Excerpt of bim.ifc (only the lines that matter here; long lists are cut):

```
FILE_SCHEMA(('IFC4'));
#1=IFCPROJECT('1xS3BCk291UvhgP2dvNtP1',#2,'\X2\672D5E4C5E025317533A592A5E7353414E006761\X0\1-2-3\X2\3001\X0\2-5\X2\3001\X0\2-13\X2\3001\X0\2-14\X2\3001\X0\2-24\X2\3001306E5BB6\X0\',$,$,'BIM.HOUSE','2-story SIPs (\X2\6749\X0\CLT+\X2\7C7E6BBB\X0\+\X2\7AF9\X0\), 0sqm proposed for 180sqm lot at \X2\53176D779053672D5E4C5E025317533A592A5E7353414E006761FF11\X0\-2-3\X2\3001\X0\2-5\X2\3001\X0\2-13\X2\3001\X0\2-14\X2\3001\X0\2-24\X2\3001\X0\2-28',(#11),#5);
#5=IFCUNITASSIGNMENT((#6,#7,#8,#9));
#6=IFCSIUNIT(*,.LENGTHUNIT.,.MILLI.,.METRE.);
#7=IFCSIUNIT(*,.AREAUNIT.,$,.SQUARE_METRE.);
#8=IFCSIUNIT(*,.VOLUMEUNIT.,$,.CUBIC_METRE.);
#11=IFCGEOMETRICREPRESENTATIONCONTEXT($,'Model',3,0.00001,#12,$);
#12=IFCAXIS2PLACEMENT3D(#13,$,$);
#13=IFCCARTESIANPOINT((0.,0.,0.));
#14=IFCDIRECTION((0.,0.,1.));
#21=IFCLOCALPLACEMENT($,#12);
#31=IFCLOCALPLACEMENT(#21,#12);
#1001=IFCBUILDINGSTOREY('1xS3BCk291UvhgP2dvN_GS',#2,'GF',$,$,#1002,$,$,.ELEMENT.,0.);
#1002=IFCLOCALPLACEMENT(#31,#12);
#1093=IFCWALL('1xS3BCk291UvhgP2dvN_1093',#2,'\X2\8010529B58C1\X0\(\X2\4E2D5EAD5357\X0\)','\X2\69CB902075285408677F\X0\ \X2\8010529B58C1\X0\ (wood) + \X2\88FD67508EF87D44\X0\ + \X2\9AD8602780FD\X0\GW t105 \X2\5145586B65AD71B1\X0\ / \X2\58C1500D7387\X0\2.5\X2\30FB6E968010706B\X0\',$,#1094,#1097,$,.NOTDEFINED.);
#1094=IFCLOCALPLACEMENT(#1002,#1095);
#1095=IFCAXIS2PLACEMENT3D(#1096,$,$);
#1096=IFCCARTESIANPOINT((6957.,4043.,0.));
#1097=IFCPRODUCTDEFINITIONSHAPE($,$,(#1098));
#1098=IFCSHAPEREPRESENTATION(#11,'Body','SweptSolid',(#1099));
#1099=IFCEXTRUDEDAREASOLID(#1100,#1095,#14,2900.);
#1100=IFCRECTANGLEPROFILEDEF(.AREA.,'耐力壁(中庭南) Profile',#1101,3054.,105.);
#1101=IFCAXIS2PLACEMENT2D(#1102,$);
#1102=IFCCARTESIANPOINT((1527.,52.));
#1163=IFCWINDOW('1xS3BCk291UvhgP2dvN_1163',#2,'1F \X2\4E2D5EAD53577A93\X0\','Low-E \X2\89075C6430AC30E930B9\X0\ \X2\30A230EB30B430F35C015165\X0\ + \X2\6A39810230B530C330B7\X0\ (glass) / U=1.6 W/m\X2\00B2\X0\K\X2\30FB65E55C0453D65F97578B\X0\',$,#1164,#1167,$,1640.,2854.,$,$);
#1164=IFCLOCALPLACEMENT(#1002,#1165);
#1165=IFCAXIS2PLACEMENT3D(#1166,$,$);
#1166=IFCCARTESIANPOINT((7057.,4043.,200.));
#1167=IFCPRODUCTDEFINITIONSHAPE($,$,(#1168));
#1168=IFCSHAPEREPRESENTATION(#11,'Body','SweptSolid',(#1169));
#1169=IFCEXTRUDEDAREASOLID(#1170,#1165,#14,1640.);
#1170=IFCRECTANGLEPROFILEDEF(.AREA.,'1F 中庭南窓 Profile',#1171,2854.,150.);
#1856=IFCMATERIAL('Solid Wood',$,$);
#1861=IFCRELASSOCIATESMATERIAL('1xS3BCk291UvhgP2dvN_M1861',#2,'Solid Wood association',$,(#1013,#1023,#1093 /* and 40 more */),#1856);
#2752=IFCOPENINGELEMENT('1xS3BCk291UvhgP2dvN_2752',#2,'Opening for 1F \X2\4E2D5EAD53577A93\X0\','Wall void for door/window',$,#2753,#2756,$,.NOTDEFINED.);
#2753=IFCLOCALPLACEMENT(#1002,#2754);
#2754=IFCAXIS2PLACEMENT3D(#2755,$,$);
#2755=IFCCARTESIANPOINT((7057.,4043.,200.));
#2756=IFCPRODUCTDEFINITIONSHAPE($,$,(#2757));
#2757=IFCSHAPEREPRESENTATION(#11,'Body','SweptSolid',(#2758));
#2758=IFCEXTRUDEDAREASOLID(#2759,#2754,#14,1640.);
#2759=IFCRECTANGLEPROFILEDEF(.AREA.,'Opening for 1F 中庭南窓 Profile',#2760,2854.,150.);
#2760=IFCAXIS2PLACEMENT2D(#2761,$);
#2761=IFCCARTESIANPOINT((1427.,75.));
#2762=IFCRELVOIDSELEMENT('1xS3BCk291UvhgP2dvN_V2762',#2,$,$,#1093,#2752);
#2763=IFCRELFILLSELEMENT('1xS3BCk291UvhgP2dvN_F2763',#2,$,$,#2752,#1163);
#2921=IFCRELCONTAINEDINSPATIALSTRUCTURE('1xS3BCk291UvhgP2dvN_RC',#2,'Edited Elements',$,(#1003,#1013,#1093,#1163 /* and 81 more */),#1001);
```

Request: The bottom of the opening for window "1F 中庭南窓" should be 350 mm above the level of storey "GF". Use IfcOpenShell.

```python
import numpy as np
import ifcopenshell
import ifcopenshell.api.geometry
import ifcopenshell.geom
import ifcopenshell.util.element
import ifcopenshell.util.placement
import ifcopenshell.util.shape
import ifcopenshell.util.unit

model = ifcopenshell.open("bim.ifc")
unit_scale = ifcopenshell.util.unit.calculate_unit_scale(model)

window = model.by_id(1163)
opening = window.FillsVoids[0].RelatingOpeningElement
storey = ifcopenshell.util.element.get_container(window, ifc_class="IfcBuildingStorey")
level = ifcopenshell.util.placement.get_local_placement(storey.ObjectPlacement)[2, 3]

# The opening's origin need not be at the sill, so measure its lowest point.
shape = ifcopenshell.geom.create_shape(ifcopenshell.geom.settings(), opening)
bottom = ifcopenshell.util.shape.get_shape_bottom_elevation(shape, shape.geometry) / unit_scale
dz = level + 0.35 / unit_scale - bottom

shift = np.array([0.0, 0.0, dz])
# The window is not placed relative to its opening, so move both.
for product in (opening, window):
    matrix = ifcopenshell.util.placement.get_local_placement(product.ObjectPlacement)
    matrix[:3, 3] += shift
    ifcopenshell.api.geometry.edit_object_placement(model, product=product, matrix=matrix, is_si=False)

print(f"moved by {dz * unit_scale:+.3f} m")

model.write("bim_v2.ifc")
```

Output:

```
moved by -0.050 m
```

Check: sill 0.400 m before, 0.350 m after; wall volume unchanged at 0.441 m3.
